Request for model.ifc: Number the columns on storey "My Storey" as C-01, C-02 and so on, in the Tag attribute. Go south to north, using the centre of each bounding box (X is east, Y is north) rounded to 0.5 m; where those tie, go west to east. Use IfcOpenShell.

First a look at what the model holds.

```python
import ifcopenshell
import ifcopenshell.util.element
import ifcopenshell.util.placement

model = ifcopenshell.open("model.ifc")
print(model.schema)
storey = next(s for s in model.by_type("IfcBuildingStorey") if s.Name == "My Storey")
columns = [e for e in ifcopenshell.util.element.get_decomposition(storey) if e.is_a("IfcColumn")]
for e in sorted(columns, key=lambda e: e.id()):
    origin = ifcopenshell.util.placement.get_local_placement(e.ObjectPlacement)[:3, 3]
    print(e.id(), e.Tag, e.Name, origin.round(2) + 0.0, sep=" | ")
```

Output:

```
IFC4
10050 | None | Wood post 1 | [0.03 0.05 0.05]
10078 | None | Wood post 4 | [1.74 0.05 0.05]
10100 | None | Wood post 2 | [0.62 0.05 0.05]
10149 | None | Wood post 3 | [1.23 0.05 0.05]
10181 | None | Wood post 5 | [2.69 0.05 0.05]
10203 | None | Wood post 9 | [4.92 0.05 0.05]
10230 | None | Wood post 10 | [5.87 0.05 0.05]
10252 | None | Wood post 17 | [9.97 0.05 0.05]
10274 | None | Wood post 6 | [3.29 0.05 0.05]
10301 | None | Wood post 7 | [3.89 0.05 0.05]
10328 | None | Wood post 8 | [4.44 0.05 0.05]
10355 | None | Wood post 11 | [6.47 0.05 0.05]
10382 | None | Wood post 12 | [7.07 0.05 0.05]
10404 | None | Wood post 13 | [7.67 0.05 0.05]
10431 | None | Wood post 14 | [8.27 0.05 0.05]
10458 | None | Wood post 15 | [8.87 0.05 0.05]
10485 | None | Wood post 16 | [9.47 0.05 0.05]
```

```python
import ifcopenshell
import ifcopenshell.geom
import ifcopenshell.util.element
import ifcopenshell.util.shape

model = ifcopenshell.open("model.ifc")
settings = ifcopenshell.geom.settings()
settings.set("use-world-coords", True)


def centre(element):
    shape = ifcopenshell.geom.create_shape(settings, element)
    return ifcopenshell.util.shape.get_bbox_centroid(shape.geometry)


storey = next(s for s in model.by_type("IfcBuildingStorey") if s.Name == "My Storey")
columns = [e for e in ifcopenshell.util.element.get_decomposition(storey) if e.is_a("IfcColumn")]

# Insertion points can sit at a corner or the storey origin, so sort by the geometry (in metres).
centres = {e: centre(e) for e in columns}
columns.sort(key=lambda e: (round(centres[e][1] / 0.5), centres[e][0]))

for i, e in enumerate(columns, start=1):
    number = f"C-{i:02d}"
    e.Tag = number
    print(e.id(), number)

model.write("model_updated.ifc")
```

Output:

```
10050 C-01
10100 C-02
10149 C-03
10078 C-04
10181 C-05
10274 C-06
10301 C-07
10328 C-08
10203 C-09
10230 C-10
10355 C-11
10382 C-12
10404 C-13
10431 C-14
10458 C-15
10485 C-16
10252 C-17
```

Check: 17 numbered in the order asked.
